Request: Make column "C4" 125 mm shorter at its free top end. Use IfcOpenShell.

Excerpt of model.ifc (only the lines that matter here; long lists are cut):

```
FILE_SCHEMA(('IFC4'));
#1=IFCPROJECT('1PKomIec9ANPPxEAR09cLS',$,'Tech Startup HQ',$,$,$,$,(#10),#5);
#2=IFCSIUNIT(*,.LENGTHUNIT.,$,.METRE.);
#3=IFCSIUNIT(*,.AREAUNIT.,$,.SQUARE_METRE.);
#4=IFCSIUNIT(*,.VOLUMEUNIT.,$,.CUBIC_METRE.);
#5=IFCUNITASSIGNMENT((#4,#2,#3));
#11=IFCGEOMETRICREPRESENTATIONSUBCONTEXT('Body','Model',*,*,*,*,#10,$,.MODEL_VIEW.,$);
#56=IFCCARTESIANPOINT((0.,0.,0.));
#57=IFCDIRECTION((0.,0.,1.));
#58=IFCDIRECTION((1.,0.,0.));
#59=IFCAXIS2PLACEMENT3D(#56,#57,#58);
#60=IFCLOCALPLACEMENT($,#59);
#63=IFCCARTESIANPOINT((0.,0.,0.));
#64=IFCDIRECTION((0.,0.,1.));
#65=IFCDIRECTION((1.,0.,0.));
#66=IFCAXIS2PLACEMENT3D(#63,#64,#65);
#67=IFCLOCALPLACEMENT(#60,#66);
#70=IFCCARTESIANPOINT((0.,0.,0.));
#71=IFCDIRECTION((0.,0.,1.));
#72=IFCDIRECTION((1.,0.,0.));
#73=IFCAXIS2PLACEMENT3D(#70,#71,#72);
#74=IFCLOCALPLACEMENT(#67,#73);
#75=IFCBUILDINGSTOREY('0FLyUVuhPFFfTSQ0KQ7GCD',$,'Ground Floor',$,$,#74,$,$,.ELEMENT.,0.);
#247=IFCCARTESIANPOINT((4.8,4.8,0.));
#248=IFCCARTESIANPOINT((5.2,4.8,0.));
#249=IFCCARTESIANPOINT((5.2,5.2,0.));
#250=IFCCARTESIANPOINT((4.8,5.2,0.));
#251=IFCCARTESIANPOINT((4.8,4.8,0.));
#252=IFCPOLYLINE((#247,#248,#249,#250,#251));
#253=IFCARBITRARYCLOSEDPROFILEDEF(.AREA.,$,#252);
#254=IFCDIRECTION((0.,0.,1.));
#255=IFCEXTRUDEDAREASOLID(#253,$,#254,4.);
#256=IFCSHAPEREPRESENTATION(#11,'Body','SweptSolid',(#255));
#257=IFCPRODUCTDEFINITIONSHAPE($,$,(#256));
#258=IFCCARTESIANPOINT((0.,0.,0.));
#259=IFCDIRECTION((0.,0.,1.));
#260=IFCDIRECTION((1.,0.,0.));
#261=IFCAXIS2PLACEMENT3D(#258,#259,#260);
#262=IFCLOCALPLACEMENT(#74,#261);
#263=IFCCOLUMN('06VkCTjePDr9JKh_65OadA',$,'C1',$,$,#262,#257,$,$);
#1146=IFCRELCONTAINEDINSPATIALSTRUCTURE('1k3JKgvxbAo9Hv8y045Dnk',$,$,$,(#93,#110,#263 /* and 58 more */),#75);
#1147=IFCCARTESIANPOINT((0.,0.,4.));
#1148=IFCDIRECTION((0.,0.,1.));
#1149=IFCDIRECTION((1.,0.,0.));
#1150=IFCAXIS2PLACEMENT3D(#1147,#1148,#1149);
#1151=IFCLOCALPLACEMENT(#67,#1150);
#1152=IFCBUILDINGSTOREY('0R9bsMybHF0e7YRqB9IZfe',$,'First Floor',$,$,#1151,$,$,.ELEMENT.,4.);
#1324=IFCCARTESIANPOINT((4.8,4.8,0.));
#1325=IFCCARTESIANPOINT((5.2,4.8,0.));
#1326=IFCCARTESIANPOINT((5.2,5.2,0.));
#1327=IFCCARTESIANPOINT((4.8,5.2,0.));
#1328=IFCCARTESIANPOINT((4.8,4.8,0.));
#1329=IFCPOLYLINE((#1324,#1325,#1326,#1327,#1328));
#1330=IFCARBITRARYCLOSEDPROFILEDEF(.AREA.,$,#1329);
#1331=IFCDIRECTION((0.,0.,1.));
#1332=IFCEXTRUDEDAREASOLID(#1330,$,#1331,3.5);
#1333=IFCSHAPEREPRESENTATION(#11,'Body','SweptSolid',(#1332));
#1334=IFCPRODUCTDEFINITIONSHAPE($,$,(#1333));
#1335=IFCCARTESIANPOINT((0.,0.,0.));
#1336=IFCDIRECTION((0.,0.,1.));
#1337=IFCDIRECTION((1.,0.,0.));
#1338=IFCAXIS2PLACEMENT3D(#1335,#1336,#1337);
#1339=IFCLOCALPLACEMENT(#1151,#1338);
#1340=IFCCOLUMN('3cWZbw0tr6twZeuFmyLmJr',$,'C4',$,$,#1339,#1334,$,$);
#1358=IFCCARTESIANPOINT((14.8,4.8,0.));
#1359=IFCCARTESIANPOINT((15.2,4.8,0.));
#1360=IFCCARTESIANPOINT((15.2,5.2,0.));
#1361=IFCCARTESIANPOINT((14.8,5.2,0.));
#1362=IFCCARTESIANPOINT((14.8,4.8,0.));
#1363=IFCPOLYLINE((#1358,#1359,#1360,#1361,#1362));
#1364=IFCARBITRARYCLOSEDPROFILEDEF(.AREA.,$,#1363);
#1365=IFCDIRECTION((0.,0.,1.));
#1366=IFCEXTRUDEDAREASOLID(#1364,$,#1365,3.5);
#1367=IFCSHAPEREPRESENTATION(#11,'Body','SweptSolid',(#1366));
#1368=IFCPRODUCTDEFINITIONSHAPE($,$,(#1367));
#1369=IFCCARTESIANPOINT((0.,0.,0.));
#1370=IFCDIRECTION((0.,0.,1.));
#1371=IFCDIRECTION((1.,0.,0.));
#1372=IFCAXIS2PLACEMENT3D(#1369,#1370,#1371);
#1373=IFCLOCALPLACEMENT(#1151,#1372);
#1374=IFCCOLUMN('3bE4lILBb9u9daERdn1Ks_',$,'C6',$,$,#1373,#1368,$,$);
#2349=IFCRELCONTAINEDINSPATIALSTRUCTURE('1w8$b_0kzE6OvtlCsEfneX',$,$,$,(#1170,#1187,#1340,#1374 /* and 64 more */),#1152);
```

```python
import ifcopenshell
import ifcopenshell.util.representation

model = ifcopenshell.open("model.ifc")

member = model.by_guid("3cWZbw0tr6twZeuFmyLmJr")
change = -0.125

# The extrusion runs towards the end named, so only its depth changes.
body = ifcopenshell.util.representation.get_representation(member, "Model", "Body")
solid = body.Items[0]
old_length = solid.Depth
solid.Depth += change

print(f"length {old_length:g} -> {solid.Depth:g}")

model.write("model_v2.ifc")
```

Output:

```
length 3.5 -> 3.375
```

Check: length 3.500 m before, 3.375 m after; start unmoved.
